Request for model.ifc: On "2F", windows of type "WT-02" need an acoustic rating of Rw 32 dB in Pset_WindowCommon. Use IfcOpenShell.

First a look at what the model holds.

```python
import ifcopenshell
import ifcopenshell.util.element

model = ifcopenshell.open("model.ifc")
print(model.schema)
storey = next(s for s in model.by_type("IfcBuildingStorey") if s.Name == "2F")
windows = [e for e in ifcopenshell.util.element.get_decomposition(storey) if e.is_a("IfcWindow")]
seen = {}
for e in windows:
    element_type = ifcopenshell.util.element.get_type(e)
    key = (element_type.Name if element_type != e and element_type else None, ifcopenshell.util.element.get_pset(e, "Pset_WindowCommon", "AcousticRating"))
    seen[key] = seen.get(key, 0) + 1
for (name, value), count in sorted(seen.items(), key=str):
    print(count, "x", name, "|", value)
```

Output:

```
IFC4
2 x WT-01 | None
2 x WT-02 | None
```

```python
import ifcopenshell
import ifcopenshell.api.pset
import ifcopenshell.util.element

model = ifcopenshell.open("model.ifc")

storey = next(s for s in model.by_type("IfcBuildingStorey") if s.Name == "2F")
windows = [e for e in ifcopenshell.util.element.get_decomposition(storey) if e.is_a("IfcWindow")]

count = 0
for e in windows:
    element_type = ifcopenshell.util.element.get_type(e)
    if element_type in (None, e) or element_type.Name != "WT-02":
        continue
    # add_pset returns the element's existing set when there is one.
    pset = ifcopenshell.api.pset.add_pset(model, product=e, name="Pset_WindowCommon")
    ifcopenshell.api.pset.edit_pset(model, pset=pset, properties={"AcousticRating": "Rw 32 dB"})
    count += 1

print(count, "windows updated")

model.write("model_updated.ifc")
```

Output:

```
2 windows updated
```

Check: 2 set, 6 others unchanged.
